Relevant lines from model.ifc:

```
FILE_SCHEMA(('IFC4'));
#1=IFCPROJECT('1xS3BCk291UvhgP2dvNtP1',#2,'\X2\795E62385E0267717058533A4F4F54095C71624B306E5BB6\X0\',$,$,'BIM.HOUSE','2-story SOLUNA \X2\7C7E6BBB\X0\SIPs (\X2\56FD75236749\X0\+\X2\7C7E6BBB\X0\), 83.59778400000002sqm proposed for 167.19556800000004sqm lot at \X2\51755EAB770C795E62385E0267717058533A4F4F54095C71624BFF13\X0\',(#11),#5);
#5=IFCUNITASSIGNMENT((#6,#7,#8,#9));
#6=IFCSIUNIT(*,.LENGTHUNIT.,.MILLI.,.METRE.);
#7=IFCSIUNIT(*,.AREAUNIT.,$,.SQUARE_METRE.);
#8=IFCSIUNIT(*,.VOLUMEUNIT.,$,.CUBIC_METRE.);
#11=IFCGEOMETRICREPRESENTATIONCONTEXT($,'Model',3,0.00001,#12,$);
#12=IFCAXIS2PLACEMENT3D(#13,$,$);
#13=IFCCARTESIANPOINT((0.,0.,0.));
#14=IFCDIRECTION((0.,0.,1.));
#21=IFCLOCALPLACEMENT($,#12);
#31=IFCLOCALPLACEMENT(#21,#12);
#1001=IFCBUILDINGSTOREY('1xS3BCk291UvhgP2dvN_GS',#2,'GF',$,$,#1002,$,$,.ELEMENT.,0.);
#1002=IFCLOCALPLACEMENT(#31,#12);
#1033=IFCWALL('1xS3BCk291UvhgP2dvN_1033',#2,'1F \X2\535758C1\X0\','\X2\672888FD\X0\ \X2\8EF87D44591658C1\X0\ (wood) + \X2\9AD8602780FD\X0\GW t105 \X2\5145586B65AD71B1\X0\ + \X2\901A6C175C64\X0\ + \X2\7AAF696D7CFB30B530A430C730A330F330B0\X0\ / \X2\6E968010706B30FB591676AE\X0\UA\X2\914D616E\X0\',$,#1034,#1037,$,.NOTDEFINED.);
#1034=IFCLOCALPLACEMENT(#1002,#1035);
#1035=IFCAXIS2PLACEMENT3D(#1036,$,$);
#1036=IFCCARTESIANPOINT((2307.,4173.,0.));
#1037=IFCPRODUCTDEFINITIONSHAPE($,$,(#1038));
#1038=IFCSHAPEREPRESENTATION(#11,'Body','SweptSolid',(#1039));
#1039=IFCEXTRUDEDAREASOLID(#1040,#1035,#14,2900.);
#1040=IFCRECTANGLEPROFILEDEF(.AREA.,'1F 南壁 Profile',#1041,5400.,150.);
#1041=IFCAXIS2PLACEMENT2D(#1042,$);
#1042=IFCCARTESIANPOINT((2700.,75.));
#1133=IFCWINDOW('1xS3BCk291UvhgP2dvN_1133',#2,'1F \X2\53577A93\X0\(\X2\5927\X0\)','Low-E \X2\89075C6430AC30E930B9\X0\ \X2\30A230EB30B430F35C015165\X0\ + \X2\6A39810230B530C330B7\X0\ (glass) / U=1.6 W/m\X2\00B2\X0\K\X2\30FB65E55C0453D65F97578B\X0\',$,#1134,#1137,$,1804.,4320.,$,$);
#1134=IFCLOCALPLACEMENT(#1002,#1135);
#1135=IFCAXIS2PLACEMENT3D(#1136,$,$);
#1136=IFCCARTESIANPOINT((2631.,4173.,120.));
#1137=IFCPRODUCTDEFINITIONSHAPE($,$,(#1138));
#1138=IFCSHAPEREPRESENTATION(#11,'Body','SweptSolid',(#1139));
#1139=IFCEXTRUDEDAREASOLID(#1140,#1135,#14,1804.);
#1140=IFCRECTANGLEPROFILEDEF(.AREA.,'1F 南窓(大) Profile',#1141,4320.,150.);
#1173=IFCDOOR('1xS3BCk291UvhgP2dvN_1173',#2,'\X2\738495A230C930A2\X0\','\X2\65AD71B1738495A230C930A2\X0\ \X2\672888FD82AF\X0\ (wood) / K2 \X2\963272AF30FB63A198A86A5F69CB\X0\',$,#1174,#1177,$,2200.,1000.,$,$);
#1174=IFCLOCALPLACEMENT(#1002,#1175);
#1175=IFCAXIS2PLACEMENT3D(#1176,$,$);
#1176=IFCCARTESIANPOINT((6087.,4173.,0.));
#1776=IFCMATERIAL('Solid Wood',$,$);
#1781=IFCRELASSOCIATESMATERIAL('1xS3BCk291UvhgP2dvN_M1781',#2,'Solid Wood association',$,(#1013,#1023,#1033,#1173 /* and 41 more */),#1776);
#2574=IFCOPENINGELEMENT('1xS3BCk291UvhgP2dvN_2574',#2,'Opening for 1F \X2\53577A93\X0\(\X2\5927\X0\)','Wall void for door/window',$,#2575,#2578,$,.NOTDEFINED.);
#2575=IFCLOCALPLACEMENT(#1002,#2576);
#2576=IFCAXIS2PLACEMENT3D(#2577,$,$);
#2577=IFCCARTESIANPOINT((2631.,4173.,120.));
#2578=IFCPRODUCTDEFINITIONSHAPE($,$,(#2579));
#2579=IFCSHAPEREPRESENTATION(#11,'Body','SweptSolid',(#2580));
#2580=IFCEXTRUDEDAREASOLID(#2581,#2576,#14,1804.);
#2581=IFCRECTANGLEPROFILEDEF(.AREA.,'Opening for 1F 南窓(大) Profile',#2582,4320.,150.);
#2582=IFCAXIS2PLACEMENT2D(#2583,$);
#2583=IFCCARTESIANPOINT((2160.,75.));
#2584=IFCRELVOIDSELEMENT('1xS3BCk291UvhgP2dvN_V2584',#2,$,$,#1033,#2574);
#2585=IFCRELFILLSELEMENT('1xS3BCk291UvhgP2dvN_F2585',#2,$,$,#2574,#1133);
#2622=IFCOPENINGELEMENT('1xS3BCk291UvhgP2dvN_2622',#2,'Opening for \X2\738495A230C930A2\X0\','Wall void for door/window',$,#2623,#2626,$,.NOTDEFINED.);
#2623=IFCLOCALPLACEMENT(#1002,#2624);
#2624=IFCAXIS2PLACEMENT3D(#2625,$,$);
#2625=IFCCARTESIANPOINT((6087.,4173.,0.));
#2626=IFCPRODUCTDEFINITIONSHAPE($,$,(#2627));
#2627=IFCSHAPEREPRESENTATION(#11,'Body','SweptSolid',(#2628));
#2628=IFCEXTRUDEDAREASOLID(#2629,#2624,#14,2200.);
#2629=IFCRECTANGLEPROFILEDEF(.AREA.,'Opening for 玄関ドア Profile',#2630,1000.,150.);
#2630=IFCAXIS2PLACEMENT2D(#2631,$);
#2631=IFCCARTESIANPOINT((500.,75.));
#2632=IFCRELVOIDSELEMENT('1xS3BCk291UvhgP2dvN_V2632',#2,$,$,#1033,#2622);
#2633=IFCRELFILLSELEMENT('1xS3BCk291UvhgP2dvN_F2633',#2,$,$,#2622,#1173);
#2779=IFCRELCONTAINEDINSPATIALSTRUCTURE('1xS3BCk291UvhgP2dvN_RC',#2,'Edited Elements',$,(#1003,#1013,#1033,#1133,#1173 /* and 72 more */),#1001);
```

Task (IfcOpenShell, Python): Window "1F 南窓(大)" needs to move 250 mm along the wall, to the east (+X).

```python
import ifcopenshell
import ifcopenshell.api.geometry
import ifcopenshell.util.placement

model = ifcopenshell.open("model.ifc")

window = model.by_guid("1xS3BCk291UvhgP2dvN_1133")
opening = window.FillsVoids[0].RelatingOpeningElement
wall = opening.VoidsElements[0].RelatingBuildingElement

wall_matrix = ifcopenshell.util.placement.get_local_placement(wall.ObjectPlacement)
shift = wall_matrix[:3, 0] * 250.0
before = ifcopenshell.util.placement.get_local_placement(window.ObjectPlacement)[:3, 3].copy()

# The window is not placed relative to its opening, so move both.
for product in (opening, window):
    matrix = ifcopenshell.util.placement.get_local_placement(product.ObjectPlacement)
    matrix[:3, 3] += shift
    ifcopenshell.api.geometry.edit_object_placement(model, product=product, matrix=matrix, is_si=False)

after = ifcopenshell.util.placement.get_local_placement(window.ObjectPlacement)[:3, 3]
print("window moved by", (after - before).round(3) + 0.0)

model.write("model_rev.ifc")
```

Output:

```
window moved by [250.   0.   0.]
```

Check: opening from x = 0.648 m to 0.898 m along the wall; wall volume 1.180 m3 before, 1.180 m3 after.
